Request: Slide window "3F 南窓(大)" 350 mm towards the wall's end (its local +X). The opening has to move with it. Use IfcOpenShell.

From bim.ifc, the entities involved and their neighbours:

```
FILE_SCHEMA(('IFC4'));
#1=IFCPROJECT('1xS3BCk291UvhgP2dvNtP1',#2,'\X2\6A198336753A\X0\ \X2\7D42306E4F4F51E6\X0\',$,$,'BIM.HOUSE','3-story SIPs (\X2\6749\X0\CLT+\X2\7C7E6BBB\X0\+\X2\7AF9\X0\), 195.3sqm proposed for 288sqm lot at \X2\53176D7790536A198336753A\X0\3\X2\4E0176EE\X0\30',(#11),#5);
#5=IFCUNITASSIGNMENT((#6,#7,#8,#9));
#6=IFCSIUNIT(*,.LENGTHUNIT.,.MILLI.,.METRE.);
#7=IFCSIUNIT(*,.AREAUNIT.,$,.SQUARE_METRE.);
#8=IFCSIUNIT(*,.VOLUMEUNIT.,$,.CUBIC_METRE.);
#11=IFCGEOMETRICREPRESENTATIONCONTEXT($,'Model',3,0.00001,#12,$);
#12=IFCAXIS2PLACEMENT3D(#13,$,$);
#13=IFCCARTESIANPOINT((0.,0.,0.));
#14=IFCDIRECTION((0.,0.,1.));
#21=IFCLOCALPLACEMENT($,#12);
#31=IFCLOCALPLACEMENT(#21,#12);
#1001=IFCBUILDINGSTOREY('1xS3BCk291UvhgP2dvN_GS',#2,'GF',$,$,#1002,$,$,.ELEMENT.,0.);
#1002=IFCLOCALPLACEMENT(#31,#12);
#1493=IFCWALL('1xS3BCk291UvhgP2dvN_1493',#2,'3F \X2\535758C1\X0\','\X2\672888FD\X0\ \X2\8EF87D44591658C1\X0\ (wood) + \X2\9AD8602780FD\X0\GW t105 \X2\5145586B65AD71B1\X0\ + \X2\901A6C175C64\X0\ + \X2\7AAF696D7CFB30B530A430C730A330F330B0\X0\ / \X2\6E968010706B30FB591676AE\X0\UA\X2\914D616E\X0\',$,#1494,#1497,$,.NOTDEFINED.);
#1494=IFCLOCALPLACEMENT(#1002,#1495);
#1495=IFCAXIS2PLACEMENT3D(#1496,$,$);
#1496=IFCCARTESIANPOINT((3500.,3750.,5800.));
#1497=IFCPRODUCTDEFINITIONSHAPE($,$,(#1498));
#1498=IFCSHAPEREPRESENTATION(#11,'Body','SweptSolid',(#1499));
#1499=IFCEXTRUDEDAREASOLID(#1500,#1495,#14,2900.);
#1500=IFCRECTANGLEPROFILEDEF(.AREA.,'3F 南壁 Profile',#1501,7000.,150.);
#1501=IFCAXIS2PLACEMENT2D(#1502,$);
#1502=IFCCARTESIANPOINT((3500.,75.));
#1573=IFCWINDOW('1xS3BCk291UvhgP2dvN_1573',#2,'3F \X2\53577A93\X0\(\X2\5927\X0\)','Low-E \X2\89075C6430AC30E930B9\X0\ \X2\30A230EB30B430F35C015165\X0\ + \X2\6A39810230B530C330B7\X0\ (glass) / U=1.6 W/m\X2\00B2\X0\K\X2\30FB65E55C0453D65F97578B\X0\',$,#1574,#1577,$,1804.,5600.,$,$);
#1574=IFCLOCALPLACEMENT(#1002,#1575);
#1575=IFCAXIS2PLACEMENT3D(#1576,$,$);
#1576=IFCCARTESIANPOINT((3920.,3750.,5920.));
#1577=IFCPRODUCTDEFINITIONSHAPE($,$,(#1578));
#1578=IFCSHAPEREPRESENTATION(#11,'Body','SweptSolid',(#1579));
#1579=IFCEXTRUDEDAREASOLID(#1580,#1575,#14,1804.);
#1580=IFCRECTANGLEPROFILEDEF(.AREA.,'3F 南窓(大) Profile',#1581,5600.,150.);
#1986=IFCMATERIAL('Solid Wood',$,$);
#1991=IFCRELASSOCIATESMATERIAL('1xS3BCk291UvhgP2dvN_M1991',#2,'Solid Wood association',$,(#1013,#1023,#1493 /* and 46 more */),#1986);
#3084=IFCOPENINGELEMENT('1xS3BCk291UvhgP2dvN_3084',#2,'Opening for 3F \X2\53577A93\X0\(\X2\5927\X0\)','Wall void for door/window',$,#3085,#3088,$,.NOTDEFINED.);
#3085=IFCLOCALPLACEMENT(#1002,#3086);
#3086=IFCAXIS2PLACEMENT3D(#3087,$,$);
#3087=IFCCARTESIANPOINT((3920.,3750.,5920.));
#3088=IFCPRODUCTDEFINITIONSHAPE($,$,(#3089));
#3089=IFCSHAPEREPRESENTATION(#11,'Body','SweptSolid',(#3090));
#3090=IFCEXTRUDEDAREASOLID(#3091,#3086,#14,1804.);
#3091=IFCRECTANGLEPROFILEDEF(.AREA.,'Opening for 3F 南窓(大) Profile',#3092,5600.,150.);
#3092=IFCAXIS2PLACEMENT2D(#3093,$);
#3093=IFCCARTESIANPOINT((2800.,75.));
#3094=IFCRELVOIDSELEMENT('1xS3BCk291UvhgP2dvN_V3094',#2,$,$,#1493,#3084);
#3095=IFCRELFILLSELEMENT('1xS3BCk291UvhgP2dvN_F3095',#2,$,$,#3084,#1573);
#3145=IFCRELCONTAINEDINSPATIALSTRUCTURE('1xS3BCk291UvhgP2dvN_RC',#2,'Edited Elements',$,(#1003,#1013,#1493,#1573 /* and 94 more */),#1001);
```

```python
import ifcopenshell
import ifcopenshell.api.geometry
import ifcopenshell.util.placement
import ifcopenshell.util.unit

model = ifcopenshell.open("bim.ifc")
unit_scale = ifcopenshell.util.unit.calculate_unit_scale(model)

window = model.by_guid("1xS3BCk291UvhgP2dvN_1573")
opening = window.FillsVoids[0].RelatingOpeningElement
wall = opening.VoidsElements[0].RelatingBuildingElement

wall_matrix = ifcopenshell.util.placement.get_local_placement(wall.ObjectPlacement)
shift = wall_matrix[:3, 0] * 0.35 / unit_scale
before = ifcopenshell.util.placement.get_local_placement(window.ObjectPlacement)[:3, 3].copy()

# The window is not placed relative to its opening, so move both.
for product in (opening, window):
    matrix = ifcopenshell.util.placement.get_local_placement(product.ObjectPlacement)
    matrix[:3, 3] += shift
    ifcopenshell.api.geometry.edit_object_placement(model, product=product, matrix=matrix, is_si=False)

after = ifcopenshell.util.placement.get_local_placement(window.ObjectPlacement)[:3, 3]
print("window moved by", (after - before).round(3) + 0.0)

model.write("bim-out.ifc")
```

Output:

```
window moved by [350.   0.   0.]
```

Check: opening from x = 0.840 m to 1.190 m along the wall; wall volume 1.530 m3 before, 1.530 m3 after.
